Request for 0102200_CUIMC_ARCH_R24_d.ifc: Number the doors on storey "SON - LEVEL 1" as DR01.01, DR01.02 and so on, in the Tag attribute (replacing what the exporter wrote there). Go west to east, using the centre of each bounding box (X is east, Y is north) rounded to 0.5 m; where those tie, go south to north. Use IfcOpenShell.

First a look at what the model holds.

```python
import ifcopenshell
import ifcopenshell.util.element
import ifcopenshell.util.placement

model = ifcopenshell.open("0102200_CUIMC_ARCH_R24_d.ifc")
print(model.schema)
storey = next(s for s in model.by_type("IfcBuildingStorey") if s.Name == "SON - LEVEL 1")
doors = [e for e in ifcopenshell.util.element.get_decomposition(storey) if e.is_a("IfcDoor")]
for e in sorted(doors, key=lambda e: e.id()):
    origin = ifcopenshell.util.placement.get_local_placement(e.ObjectPlacement)[:3, 3]
    print(e.id(), e.Tag, e.Name, origin.round(2) + 0.0, sep=" | ")
```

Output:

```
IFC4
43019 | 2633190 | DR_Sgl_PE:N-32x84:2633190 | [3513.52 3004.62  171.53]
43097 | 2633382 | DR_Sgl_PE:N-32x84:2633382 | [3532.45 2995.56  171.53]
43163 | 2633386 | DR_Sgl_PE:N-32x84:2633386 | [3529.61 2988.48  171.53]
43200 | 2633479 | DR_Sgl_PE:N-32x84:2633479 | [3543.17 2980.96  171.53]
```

```python
import ifcopenshell
import ifcopenshell.geom
import ifcopenshell.util.element
import ifcopenshell.util.shape

model = ifcopenshell.open("0102200_CUIMC_ARCH_R24_d.ifc")
settings = ifcopenshell.geom.settings()
settings.set("use-world-coords", True)


def centre(element):
    shape = ifcopenshell.geom.create_shape(settings, element)
    return ifcopenshell.util.shape.get_bbox_centroid(shape.geometry)


storey = next(s for s in model.by_type("IfcBuildingStorey") if s.Name == "SON - LEVEL 1")
doors = [e for e in ifcopenshell.util.element.get_decomposition(storey) if e.is_a("IfcDoor")]

# Insertion points can sit at a corner or the storey origin, so sort by the geometry (in metres).
centres = {e: centre(e) for e in doors}
doors.sort(key=lambda e: (round(centres[e][0] / 0.5), centres[e][1]))

for i, e in enumerate(doors, start=1):
    number = f"DR01.{i:02d}"
    e.Tag = number
    print(e.id(), number)

model.write("0102200_CUIMC_ARCH_R24_d_v2.ifc")
```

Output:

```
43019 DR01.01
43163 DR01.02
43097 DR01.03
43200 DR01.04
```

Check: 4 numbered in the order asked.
